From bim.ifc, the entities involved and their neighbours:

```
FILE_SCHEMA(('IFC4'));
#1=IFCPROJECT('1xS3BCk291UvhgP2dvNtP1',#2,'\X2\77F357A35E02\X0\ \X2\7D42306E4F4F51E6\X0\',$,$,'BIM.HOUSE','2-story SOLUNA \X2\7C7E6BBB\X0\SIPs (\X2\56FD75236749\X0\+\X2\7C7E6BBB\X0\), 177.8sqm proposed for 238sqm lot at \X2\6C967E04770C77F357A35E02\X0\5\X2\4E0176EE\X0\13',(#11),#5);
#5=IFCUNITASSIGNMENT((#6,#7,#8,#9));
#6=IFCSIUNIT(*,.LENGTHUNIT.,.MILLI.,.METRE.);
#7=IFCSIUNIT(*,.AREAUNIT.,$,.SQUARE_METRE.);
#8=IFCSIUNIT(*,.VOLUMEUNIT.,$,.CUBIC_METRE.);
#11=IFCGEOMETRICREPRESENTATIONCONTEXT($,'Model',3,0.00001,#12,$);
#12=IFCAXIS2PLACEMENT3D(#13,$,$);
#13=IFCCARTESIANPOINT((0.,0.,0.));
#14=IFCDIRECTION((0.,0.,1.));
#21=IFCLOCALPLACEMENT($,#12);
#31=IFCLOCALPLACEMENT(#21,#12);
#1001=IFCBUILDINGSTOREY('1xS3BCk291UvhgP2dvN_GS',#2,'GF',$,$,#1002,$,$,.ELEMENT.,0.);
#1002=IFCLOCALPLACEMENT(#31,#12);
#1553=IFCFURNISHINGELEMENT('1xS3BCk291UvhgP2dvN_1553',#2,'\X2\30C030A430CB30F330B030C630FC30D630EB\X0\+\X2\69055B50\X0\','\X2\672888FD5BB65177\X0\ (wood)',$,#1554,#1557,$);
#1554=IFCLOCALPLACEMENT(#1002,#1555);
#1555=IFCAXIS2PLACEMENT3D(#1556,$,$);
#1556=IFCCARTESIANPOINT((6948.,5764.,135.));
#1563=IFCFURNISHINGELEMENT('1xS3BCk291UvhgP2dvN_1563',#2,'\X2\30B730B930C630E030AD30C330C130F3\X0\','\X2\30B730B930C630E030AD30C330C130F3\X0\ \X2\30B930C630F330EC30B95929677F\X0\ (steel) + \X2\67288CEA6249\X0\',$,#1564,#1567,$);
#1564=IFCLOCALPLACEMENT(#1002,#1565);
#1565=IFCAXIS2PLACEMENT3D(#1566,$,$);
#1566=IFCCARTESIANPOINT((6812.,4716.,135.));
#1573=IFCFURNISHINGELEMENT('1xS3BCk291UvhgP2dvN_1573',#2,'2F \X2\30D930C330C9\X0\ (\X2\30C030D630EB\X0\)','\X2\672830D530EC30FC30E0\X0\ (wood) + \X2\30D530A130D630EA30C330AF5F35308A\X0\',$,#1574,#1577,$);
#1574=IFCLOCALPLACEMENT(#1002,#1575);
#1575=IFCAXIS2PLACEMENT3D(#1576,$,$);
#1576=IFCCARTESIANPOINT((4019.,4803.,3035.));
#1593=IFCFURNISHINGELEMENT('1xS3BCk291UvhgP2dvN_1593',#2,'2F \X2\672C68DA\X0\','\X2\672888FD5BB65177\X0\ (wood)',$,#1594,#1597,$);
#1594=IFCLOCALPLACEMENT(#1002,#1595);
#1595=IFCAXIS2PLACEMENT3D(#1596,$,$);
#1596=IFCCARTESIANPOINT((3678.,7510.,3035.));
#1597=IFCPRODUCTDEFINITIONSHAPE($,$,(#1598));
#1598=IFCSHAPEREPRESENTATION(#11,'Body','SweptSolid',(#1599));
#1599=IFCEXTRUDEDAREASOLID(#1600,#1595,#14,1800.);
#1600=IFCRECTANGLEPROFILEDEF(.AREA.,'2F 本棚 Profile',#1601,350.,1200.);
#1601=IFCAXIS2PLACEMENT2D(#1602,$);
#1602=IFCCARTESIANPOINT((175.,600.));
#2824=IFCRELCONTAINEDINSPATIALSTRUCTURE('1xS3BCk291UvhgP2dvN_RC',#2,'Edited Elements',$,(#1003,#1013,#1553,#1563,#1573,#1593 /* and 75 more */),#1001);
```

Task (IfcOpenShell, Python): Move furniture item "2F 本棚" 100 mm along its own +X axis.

```python
import ifcopenshell
import ifcopenshell.api.geometry
import ifcopenshell.util.placement

model = ifcopenshell.open("bim.ifc")

item = model.by_guid("1xS3BCk291UvhgP2dvN_1593")
matrix = ifcopenshell.util.placement.get_local_placement(item.ObjectPlacement)
matrix[:3, 3] += matrix[:3, 0] * 100.0
ifcopenshell.api.geometry.edit_object_placement(model, product=item, matrix=matrix, is_si=False)

print(ifcopenshell.util.placement.get_local_placement(item.ObjectPlacement).round(3) + 0.0)

model.write("bim_rev.ifc")
```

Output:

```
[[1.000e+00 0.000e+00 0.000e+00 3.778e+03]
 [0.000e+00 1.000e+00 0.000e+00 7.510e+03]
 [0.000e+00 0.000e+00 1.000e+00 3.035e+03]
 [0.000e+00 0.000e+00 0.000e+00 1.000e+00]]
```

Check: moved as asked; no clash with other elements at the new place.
